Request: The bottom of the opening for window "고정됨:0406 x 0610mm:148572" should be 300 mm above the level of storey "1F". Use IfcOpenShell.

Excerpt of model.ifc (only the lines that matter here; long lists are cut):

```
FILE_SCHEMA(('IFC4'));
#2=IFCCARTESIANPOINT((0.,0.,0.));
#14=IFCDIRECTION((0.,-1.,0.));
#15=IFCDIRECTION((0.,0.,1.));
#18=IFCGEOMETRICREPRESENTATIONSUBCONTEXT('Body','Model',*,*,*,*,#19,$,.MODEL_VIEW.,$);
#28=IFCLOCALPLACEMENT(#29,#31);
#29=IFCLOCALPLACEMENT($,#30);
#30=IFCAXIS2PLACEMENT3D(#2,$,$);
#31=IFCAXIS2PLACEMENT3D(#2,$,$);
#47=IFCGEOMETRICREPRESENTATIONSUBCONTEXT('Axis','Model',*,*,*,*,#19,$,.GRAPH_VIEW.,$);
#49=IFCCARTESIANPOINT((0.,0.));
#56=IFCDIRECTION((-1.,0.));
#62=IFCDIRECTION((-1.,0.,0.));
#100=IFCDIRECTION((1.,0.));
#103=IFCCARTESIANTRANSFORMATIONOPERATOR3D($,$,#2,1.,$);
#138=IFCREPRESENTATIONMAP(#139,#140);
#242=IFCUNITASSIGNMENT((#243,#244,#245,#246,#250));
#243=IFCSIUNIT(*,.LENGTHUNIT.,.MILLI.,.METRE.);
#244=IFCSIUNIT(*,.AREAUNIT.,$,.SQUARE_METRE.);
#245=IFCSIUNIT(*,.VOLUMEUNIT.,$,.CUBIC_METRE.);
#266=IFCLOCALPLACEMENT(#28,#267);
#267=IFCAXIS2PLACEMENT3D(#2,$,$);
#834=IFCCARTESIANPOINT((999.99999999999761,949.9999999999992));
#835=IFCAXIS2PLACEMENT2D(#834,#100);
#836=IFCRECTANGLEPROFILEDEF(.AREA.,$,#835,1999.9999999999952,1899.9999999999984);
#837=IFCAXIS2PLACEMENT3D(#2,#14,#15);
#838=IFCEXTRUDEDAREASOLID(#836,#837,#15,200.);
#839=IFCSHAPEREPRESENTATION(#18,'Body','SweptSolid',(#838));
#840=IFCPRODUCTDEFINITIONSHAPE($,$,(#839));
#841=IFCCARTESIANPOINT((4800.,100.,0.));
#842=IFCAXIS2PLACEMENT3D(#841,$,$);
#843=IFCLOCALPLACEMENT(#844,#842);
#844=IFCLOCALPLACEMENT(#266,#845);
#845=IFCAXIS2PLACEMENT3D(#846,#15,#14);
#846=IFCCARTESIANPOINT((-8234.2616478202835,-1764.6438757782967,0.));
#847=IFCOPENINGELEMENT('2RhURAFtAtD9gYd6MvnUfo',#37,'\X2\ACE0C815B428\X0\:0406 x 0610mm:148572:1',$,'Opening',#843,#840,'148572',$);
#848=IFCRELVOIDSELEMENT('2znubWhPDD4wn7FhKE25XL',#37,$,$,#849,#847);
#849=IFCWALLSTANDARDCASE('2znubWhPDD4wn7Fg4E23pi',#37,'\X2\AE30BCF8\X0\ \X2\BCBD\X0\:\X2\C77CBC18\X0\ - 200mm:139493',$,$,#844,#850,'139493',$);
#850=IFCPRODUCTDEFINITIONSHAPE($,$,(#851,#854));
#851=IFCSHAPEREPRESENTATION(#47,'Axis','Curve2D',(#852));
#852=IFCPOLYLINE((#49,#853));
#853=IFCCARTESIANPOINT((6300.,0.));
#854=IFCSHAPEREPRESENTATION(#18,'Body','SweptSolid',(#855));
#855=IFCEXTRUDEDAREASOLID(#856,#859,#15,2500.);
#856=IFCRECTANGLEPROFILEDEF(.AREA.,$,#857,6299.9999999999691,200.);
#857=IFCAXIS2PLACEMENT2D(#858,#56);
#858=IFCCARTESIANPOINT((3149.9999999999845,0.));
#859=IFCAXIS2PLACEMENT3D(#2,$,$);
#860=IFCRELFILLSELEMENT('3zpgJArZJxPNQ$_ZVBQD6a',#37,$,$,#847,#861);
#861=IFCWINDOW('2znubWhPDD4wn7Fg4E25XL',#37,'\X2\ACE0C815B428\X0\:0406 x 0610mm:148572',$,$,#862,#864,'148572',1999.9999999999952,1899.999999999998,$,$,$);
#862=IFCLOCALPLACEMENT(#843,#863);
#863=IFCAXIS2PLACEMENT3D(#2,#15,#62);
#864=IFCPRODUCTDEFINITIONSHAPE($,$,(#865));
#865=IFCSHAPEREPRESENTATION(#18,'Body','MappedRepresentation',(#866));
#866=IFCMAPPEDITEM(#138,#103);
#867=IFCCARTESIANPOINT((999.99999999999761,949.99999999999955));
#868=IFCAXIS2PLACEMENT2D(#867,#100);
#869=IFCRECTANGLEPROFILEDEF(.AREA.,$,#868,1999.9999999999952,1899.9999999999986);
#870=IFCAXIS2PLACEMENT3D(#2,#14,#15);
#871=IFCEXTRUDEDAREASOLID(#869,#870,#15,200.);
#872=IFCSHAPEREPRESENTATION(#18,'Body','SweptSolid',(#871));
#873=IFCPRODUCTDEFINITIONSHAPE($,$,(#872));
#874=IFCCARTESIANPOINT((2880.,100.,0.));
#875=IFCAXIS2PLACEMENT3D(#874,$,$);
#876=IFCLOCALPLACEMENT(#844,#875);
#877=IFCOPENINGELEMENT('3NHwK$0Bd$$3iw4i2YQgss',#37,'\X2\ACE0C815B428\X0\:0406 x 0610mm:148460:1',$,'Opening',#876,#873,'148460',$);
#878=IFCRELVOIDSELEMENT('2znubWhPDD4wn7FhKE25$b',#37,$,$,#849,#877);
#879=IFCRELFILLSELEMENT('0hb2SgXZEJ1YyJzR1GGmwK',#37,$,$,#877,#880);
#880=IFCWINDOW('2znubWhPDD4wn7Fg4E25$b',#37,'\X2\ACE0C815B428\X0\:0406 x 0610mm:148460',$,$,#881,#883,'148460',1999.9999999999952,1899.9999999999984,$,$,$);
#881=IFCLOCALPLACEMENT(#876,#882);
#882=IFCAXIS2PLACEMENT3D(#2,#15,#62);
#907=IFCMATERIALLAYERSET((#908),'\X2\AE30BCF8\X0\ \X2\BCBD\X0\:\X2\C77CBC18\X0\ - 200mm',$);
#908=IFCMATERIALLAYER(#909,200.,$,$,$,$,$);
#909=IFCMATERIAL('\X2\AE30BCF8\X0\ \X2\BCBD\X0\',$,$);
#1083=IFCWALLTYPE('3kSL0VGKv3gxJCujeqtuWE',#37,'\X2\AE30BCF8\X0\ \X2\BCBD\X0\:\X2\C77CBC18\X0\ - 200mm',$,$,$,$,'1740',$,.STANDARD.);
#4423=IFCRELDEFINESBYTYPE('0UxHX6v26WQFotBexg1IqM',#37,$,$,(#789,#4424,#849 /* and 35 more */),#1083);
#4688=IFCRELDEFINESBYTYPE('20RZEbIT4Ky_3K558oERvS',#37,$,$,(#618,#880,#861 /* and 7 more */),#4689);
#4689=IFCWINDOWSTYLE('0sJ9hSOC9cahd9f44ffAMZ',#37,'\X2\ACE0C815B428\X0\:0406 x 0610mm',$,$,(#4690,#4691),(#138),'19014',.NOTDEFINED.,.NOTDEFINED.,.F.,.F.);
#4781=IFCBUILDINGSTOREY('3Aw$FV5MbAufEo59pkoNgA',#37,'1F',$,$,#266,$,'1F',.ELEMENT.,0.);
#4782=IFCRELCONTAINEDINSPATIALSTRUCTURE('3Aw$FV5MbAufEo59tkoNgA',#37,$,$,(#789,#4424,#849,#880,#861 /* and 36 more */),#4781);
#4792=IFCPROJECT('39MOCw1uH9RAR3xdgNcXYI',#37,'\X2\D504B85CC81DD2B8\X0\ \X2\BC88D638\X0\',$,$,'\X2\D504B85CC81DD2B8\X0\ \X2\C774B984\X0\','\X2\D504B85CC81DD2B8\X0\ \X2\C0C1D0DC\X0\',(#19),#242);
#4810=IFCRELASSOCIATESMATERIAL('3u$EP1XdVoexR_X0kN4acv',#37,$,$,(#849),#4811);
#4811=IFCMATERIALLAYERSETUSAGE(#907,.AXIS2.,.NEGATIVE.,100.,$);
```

```python
import numpy as np
import ifcopenshell
import ifcopenshell.api.geometry
import ifcopenshell.geom
import ifcopenshell.util.element
import ifcopenshell.util.placement
import ifcopenshell.util.shape
import ifcopenshell.util.unit

model = ifcopenshell.open("model.ifc")
unit_scale = ifcopenshell.util.unit.calculate_unit_scale(model)

window = model.by_id(861)
opening = window.FillsVoids[0].RelatingOpeningElement
storey = ifcopenshell.util.element.get_container(window, ifc_class="IfcBuildingStorey")
level = ifcopenshell.util.placement.get_local_placement(storey.ObjectPlacement)[2, 3]

# The opening's origin need not be at the sill, so measure its lowest point.
shape = ifcopenshell.geom.create_shape(ifcopenshell.geom.settings(), opening)
bottom = ifcopenshell.util.shape.get_shape_bottom_elevation(shape, shape.geometry) / unit_scale
dz = level + 300.0 - bottom

shift = np.array([0.0, 0.0, dz])
# The window is placed relative to its opening, so it follows when the opening moves.
matrix = ifcopenshell.util.placement.get_local_placement(opening.ObjectPlacement)
matrix[:3, 3] += shift
ifcopenshell.api.geometry.edit_object_placement(
    model, product=opening, matrix=matrix, is_si=False, should_transform_children=True
)

print(f"moved by {dz * unit_scale:+.3f} m")

model.write("model_rev.ifc")
```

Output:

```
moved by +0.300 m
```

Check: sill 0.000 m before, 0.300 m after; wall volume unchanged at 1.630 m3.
